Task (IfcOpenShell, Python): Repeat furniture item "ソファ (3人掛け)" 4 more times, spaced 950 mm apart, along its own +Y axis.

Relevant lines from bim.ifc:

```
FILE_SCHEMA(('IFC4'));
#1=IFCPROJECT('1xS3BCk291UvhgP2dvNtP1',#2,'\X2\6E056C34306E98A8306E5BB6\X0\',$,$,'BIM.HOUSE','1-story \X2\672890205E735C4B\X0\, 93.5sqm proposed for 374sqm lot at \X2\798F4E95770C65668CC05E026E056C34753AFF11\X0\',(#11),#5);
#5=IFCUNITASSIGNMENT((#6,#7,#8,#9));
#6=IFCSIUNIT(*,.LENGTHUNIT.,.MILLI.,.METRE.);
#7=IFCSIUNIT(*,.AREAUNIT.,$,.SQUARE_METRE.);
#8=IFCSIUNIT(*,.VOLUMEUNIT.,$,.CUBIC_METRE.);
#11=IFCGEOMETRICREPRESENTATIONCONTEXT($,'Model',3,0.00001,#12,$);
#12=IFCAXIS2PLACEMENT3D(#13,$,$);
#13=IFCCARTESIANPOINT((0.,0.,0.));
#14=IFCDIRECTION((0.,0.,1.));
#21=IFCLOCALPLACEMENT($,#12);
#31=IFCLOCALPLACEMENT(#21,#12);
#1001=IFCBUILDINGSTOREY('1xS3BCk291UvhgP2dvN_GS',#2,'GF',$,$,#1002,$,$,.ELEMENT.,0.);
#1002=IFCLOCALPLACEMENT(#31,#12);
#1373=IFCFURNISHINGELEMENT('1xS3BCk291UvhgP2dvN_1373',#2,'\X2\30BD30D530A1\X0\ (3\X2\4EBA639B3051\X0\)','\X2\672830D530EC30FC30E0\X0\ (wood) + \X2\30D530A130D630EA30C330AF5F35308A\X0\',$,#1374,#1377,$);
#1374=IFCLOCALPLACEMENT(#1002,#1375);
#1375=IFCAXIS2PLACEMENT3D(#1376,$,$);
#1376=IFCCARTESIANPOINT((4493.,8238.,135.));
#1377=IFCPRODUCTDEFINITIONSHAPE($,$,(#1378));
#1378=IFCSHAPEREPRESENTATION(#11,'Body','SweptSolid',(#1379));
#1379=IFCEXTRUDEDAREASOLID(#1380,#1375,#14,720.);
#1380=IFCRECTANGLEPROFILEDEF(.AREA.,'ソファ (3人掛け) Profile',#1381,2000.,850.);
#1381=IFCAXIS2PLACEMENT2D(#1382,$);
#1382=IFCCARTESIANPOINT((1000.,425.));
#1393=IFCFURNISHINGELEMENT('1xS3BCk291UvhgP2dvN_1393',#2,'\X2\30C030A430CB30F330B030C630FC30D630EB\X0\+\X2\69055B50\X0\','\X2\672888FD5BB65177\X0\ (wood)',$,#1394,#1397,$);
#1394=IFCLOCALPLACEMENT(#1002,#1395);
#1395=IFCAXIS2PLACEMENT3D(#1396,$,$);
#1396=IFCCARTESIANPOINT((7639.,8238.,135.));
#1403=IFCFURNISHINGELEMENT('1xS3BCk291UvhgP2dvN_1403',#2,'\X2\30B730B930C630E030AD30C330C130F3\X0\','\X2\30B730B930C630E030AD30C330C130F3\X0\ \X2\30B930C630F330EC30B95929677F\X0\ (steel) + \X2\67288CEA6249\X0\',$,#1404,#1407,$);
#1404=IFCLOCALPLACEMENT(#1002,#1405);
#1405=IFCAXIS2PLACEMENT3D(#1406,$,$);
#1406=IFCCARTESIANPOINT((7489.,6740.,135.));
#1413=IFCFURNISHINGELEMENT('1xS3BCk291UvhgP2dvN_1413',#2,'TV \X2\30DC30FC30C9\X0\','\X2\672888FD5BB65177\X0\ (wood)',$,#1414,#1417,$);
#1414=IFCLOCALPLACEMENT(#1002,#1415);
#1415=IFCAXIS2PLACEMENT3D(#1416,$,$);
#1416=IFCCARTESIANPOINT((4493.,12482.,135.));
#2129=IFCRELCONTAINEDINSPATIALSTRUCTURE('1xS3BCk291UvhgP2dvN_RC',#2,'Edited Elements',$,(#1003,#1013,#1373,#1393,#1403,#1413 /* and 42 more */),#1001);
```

```python
import ifcopenshell
import ifcopenshell.api.geometry
import ifcopenshell.api.root
import ifcopenshell.util.element
import ifcopenshell.util.placement
import ifcopenshell.util.unit

model = ifcopenshell.open("bim.ifc")
unit_scale = ifcopenshell.util.unit.calculate_unit_scale(model)


def reuse_history(source, copy):
    """copy_class also copies each property set's owner history, people and application; keep the originals."""
    for rel in copy.IsDefinedBy:
        if rel.is_a("IfcRelDefinesByProperties") and (history := rel.RelatingPropertyDefinition.OwnerHistory):
            rel.RelatingPropertyDefinition.OwnerHistory = source.OwnerHistory
            ifcopenshell.util.element.remove_deep2(model, history)


source = model.by_guid("1xS3BCk291UvhgP2dvN_1373")
base = ifcopenshell.util.placement.get_local_placement(source.ObjectPlacement)
step = base[:3, 1] * 0.95 / unit_scale

for i in range(1, 5):
    copy = ifcopenshell.api.root.copy_class(model, product=source)
    copy.Representation = ifcopenshell.util.element.copy_deep(
        model, source.Representation, exclude=["IfcGeometricRepresentationContext", "IfcRepresentationMap"]
    )
    reuse_history(source, copy)
    matrix = base.copy()
    matrix[:3, 3] += i * step
    print("added at", matrix[:3, 3].round(3) + 0.0)
    ifcopenshell.api.geometry.edit_object_placement(model, product=copy, matrix=matrix, is_si=False)

model.write("bim_rev.ifc")
```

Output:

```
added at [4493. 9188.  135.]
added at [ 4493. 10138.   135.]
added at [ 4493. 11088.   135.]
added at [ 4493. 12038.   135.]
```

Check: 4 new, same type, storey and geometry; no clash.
